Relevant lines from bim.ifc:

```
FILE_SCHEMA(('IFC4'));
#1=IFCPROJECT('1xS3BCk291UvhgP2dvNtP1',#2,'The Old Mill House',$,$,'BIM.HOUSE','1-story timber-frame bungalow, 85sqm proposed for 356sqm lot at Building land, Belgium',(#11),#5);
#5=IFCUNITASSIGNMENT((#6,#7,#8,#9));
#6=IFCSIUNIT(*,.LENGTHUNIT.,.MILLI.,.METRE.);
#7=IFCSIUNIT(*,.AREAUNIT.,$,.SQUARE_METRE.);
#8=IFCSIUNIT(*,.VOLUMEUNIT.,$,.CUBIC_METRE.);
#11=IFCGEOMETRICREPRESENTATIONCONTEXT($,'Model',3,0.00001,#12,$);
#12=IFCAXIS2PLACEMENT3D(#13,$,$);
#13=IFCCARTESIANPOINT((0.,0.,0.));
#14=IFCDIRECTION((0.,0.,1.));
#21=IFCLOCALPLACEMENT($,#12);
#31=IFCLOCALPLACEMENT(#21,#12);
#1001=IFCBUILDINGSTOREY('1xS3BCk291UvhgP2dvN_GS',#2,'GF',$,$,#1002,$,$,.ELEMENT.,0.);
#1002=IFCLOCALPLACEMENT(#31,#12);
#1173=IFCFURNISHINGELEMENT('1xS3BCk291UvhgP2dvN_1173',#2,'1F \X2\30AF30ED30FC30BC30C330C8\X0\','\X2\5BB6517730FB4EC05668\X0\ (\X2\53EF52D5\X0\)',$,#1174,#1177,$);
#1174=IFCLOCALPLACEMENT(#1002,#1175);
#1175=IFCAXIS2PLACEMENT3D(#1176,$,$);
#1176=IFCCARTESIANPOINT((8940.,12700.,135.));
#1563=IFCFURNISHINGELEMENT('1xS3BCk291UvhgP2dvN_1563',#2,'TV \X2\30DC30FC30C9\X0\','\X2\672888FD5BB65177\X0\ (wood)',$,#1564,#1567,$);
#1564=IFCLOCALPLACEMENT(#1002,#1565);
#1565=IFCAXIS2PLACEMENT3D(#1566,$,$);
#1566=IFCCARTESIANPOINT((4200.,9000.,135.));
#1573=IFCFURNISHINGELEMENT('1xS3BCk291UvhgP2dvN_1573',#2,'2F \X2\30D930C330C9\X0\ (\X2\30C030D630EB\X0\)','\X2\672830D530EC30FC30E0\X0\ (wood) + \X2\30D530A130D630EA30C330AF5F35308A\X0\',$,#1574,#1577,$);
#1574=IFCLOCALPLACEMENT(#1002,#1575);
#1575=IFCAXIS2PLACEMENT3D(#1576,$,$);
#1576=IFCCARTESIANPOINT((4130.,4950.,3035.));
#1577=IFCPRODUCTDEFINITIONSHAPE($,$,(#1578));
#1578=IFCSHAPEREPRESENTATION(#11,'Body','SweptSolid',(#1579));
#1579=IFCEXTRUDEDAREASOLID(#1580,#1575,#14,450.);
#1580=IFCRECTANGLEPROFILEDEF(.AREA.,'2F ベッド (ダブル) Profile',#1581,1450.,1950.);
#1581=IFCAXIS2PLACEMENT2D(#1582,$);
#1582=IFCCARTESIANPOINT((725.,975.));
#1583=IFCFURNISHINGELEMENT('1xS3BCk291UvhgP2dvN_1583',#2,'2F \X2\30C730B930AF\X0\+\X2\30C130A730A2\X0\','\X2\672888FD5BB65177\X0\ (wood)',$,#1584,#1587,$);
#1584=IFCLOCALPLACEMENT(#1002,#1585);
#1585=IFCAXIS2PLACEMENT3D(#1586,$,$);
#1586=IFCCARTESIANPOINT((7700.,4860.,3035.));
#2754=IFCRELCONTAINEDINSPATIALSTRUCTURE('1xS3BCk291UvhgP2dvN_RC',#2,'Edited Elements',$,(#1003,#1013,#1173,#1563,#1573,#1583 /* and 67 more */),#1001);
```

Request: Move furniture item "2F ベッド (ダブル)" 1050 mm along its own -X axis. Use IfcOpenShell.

```python
import ifcopenshell
import ifcopenshell.api.geometry
import ifcopenshell.util.placement

model = ifcopenshell.open("bim.ifc")

item = model.by_guid("1xS3BCk291UvhgP2dvN_1573")
matrix = ifcopenshell.util.placement.get_local_placement(item.ObjectPlacement)
matrix[:3, 3] -= matrix[:3, 0] * 1050.0
ifcopenshell.api.geometry.edit_object_placement(model, product=item, matrix=matrix, is_si=False)

print(ifcopenshell.util.placement.get_local_placement(item.ObjectPlacement).round(3) + 0.0)

model.write("bim-out.ifc")
```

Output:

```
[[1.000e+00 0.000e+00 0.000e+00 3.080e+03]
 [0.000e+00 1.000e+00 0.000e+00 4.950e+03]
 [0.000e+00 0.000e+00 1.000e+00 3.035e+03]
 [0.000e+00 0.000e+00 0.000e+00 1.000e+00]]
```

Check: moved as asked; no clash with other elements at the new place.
